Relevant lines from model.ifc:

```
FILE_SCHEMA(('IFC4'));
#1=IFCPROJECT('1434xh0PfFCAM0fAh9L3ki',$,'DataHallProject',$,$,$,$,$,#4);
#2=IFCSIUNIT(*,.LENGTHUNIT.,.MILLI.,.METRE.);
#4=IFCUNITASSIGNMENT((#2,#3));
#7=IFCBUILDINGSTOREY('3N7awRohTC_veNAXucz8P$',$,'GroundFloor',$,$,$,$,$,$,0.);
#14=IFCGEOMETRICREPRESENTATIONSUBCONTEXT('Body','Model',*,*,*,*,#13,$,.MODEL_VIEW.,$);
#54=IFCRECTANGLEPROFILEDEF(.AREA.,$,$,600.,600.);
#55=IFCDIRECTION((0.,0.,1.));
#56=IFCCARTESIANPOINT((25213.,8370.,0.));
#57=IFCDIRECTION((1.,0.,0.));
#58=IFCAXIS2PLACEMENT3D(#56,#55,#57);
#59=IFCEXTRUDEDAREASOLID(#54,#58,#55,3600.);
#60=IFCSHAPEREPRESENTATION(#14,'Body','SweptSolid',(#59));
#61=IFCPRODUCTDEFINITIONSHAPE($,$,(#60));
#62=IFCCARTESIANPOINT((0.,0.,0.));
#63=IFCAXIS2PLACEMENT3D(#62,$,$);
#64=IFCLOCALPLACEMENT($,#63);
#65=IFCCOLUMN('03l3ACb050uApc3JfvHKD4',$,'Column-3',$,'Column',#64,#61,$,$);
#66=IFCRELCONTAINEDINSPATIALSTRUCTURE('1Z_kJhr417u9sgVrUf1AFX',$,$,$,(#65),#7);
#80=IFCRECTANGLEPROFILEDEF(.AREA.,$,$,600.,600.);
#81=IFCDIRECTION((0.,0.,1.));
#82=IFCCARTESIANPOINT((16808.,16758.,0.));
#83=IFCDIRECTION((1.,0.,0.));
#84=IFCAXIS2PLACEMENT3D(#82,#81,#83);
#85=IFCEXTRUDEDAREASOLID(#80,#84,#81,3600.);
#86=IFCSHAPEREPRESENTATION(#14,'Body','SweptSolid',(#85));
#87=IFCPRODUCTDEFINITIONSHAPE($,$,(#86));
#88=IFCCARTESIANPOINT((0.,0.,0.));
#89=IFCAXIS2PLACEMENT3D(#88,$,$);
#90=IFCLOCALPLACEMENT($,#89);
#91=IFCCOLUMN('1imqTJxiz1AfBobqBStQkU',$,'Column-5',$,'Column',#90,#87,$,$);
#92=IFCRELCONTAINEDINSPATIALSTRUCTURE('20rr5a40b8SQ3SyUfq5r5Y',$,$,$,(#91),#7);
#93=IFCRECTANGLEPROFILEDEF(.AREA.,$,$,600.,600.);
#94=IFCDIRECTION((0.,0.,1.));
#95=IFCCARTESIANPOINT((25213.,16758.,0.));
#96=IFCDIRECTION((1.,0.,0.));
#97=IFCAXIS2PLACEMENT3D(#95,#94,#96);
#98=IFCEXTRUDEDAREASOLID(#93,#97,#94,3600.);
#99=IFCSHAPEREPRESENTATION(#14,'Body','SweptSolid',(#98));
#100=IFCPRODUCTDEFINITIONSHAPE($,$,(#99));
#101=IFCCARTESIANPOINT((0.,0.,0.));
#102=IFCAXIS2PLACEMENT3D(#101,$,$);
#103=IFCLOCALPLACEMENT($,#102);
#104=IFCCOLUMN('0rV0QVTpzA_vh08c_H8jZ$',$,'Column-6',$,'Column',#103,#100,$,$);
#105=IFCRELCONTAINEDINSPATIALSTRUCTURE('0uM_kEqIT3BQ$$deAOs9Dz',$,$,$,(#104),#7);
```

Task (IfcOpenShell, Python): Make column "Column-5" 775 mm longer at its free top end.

```python
import ifcopenshell
import ifcopenshell.util.representation

model = ifcopenshell.open("model.ifc")

member = model.by_guid("1imqTJxiz1AfBobqBStQkU")
change = 775.0

# The extrusion runs towards the end named, so only its depth changes.
body = ifcopenshell.util.representation.get_representation(member, "Model", "Body")
solid = body.Items[0]
old_length = solid.Depth
solid.Depth += change

print(f"length {old_length:g} -> {solid.Depth:g}")

model.write("model_rev.ifc")
```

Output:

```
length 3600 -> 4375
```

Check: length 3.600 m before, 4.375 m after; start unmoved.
